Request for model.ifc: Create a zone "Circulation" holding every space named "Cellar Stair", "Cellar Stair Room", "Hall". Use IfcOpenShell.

First a look at what the model holds.

```python
import ifcopenshell

model = ifcopenshell.open("model.ifc")
print(model.schema)
seen = {}
for space in model.by_type("IfcSpace"):
    seen[space.LongName] = seen.get(space.LongName, 0) + 1
for name, count in sorted(seen.items(), key=str):
    print(count, "x", name)
print("zones:", [z.Name for z in model.by_type("IfcZone")][:20])
```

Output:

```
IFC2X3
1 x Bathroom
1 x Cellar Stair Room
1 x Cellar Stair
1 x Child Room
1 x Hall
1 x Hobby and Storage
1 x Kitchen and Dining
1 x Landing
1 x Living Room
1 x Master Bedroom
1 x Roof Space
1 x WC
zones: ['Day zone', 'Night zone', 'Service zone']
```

```python
import ifcopenshell
import ifcopenshell.api.group
import ifcopenshell.api.root

model = ifcopenshell.open("model.ifc")

names = {"Cellar Stair", "Cellar Stair Room", "Hall"}
spaces = [s for s in model.by_type("IfcSpace") if s.LongName in names]

zone = ifcopenshell.api.root.create_entity(model, ifc_class="IfcZone", name="Circulation")
ifcopenshell.api.group.assign_group(model, products=spaces, group=zone)
print(len(spaces), "spaces in", zone.Name)

model.write("model_edited.ifc")
```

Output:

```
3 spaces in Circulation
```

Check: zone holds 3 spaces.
